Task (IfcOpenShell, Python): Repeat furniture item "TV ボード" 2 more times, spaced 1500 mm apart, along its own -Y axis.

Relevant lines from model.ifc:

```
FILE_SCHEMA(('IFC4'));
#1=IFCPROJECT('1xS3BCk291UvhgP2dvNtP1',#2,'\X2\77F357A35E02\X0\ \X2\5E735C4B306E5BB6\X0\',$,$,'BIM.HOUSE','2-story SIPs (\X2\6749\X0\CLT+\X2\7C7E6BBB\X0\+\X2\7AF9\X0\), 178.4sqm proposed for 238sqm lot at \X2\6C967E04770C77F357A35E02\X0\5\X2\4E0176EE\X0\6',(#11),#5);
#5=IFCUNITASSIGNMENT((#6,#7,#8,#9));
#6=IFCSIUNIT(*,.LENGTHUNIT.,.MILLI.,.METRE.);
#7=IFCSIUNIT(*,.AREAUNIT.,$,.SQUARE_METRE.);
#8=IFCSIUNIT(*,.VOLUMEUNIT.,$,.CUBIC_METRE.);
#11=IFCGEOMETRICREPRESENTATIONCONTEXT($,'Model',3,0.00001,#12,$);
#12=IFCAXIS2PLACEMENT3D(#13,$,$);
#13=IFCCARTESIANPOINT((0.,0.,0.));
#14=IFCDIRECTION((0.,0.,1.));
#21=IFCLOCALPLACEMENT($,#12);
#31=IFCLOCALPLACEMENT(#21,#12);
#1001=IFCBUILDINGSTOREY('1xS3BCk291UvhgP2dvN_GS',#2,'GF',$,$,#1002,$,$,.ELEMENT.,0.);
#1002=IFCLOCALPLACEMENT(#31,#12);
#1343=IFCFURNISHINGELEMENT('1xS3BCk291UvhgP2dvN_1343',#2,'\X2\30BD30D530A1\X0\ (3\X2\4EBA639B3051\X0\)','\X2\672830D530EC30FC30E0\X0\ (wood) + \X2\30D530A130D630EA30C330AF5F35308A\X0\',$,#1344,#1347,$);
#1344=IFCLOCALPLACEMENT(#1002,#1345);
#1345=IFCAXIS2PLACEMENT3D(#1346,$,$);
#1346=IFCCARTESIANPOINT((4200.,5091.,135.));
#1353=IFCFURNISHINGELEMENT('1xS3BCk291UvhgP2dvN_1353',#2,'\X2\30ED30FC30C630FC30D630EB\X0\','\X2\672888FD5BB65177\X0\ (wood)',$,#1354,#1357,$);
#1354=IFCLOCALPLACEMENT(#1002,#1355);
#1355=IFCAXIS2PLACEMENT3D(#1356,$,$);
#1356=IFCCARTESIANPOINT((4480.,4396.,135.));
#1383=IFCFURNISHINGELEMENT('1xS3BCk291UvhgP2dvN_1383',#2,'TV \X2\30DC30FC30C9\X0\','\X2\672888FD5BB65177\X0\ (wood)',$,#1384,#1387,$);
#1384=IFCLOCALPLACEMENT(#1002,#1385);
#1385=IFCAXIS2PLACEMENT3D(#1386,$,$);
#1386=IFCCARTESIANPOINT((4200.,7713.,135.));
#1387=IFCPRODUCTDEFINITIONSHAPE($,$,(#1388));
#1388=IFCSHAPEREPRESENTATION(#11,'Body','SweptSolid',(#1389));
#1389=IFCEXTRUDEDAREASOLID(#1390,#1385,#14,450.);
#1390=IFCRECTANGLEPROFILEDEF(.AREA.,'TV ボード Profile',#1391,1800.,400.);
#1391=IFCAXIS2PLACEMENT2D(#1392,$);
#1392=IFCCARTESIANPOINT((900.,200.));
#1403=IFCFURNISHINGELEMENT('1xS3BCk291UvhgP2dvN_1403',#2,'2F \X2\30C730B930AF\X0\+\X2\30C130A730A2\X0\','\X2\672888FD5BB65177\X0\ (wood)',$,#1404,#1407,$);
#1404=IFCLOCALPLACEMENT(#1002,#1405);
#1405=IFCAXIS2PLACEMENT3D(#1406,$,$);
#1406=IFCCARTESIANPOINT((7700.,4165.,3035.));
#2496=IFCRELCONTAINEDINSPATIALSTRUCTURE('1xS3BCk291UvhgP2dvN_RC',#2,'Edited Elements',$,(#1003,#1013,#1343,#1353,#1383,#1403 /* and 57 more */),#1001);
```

```python
import ifcopenshell
import ifcopenshell.api.geometry
import ifcopenshell.api.root
import ifcopenshell.util.element
import ifcopenshell.util.placement

model = ifcopenshell.open("model.ifc")


def reuse_history(source, copy):
    """copy_class also copies each property set's owner history, people and application; keep the originals."""
    for rel in copy.IsDefinedBy:
        if rel.is_a("IfcRelDefinesByProperties") and (history := rel.RelatingPropertyDefinition.OwnerHistory):
            rel.RelatingPropertyDefinition.OwnerHistory = source.OwnerHistory
            ifcopenshell.util.element.remove_deep2(model, history)


source = model.by_id(1383)
base = ifcopenshell.util.placement.get_local_placement(source.ObjectPlacement)
step = -base[:3, 1] * 1500.0

for i in range(1, 3):
    copy = ifcopenshell.api.root.copy_class(model, product=source)
    copy.Representation = ifcopenshell.util.element.copy_deep(
        model, source.Representation, exclude=["IfcGeometricRepresentationContext", "IfcRepresentationMap"]
    )
    reuse_history(source, copy)
    matrix = base.copy()
    matrix[:3, 3] += i * step
    print("added at", matrix[:3, 3].round(3) + 0.0)
    ifcopenshell.api.geometry.edit_object_placement(model, product=copy, matrix=matrix, is_si=False)

model.write("model_updated.ifc")
```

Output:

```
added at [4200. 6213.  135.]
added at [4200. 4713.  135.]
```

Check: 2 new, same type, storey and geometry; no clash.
